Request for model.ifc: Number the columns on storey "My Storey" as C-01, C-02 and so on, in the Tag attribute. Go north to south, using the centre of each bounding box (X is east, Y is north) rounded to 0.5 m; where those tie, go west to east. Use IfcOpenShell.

First a look at what the model holds.

```python
import ifcopenshell
import ifcopenshell.util.element
import ifcopenshell.util.placement

model = ifcopenshell.open("model.ifc")
print(model.schema)
storey = next(s for s in model.by_type("IfcBuildingStorey") if s.Name == "My Storey")
columns = [e for e in ifcopenshell.util.element.get_decomposition(storey) if e.is_a("IfcColumn")]
for e in sorted(columns, key=lambda e: e.id()):
    origin = ifcopenshell.util.placement.get_local_placement(e.ObjectPlacement)[:3, 3]
    print(e.id(), e.Tag, e.Name, origin.round(2) + 0.0, sep=" | ")
```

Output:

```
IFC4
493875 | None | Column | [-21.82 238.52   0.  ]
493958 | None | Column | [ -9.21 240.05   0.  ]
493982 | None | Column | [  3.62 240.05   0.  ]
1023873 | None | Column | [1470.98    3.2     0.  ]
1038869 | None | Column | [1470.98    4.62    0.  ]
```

```python
import ifcopenshell
import ifcopenshell.geom
import ifcopenshell.util.element
import ifcopenshell.util.shape

model = ifcopenshell.open("model.ifc")
settings = ifcopenshell.geom.settings()
settings.set("use-world-coords", True)


def centre(element):
    shape = ifcopenshell.geom.create_shape(settings, element)
    return ifcopenshell.util.shape.get_bbox_centroid(shape.geometry)


storey = next(s for s in model.by_type("IfcBuildingStorey") if s.Name == "My Storey")
columns = [e for e in ifcopenshell.util.element.get_decomposition(storey) if e.is_a("IfcColumn")]

# Insertion points can sit at a corner or the storey origin, so sort by the geometry (in metres).
centres = {e: centre(e) for e in columns}
columns.sort(key=lambda e: (-round(centres[e][1] / 0.5), centres[e][0]))

for i, e in enumerate(columns, start=1):
    number = f"C-{i:02d}"
    e.Tag = number
    print(e.id(), number)

model.write("model-out.ifc")
```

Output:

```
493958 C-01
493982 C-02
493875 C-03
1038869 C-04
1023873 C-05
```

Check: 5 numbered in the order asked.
